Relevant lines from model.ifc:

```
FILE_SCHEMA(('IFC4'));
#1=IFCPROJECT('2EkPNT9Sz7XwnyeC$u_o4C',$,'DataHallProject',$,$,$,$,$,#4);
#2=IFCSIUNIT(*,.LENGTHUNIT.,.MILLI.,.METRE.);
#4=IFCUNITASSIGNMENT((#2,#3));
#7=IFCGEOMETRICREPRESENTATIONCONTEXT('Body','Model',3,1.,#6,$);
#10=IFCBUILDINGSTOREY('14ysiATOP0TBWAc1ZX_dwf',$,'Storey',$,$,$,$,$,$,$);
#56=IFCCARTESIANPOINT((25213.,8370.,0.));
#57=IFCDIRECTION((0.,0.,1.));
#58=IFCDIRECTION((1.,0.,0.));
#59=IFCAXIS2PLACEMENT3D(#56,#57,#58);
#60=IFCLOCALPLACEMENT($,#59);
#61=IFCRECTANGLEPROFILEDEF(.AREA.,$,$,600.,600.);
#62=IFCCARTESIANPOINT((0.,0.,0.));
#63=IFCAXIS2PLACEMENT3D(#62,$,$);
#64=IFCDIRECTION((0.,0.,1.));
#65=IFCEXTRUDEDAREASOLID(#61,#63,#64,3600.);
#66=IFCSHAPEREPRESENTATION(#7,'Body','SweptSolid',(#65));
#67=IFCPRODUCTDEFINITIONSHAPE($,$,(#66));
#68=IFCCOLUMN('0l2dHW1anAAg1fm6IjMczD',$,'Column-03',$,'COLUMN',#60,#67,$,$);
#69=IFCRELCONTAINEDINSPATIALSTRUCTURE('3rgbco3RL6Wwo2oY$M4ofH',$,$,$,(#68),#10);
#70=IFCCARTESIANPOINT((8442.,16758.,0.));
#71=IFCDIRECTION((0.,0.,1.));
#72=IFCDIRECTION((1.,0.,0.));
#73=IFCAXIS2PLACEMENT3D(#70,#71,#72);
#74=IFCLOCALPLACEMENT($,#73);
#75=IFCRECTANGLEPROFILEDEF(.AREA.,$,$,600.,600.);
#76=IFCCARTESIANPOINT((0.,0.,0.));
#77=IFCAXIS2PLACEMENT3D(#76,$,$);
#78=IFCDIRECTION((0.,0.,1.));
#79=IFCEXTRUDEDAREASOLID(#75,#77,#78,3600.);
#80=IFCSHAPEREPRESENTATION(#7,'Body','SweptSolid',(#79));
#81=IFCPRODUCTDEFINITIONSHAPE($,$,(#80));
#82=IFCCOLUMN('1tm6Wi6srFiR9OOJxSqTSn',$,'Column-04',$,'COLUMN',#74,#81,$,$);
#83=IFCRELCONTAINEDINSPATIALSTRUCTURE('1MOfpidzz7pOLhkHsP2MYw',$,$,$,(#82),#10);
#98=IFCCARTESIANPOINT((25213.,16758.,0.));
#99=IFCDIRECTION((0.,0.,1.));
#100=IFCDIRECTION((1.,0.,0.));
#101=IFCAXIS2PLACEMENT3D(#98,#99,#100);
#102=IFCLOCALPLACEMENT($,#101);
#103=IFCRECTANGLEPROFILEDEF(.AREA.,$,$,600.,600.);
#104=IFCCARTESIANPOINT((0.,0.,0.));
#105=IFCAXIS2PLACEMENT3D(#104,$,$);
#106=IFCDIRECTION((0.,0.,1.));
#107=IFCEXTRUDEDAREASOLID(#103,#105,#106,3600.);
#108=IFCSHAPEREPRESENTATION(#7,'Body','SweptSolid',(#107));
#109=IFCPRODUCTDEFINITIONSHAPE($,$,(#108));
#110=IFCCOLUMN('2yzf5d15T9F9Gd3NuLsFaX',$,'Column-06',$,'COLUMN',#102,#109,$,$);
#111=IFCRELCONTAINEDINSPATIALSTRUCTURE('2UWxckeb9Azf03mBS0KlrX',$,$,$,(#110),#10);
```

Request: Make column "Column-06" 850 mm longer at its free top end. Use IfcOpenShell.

```python
import ifcopenshell

model = ifcopenshell.open("model.ifc")

member = model.by_guid("2yzf5d15T9F9Gd3NuLsFaX")
change = 850.0

# The extrusion runs towards the end named, so only its depth changes.
body = next(r for r in member.Representation.Representations if r.RepresentationIdentifier == "Body")
solid = body.Items[0]
old_length = solid.Depth
solid.Depth += change

print(f"length {old_length:g} -> {solid.Depth:g}")

model.write("model_v2.ifc")
```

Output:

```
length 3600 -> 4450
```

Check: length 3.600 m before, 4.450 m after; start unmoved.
